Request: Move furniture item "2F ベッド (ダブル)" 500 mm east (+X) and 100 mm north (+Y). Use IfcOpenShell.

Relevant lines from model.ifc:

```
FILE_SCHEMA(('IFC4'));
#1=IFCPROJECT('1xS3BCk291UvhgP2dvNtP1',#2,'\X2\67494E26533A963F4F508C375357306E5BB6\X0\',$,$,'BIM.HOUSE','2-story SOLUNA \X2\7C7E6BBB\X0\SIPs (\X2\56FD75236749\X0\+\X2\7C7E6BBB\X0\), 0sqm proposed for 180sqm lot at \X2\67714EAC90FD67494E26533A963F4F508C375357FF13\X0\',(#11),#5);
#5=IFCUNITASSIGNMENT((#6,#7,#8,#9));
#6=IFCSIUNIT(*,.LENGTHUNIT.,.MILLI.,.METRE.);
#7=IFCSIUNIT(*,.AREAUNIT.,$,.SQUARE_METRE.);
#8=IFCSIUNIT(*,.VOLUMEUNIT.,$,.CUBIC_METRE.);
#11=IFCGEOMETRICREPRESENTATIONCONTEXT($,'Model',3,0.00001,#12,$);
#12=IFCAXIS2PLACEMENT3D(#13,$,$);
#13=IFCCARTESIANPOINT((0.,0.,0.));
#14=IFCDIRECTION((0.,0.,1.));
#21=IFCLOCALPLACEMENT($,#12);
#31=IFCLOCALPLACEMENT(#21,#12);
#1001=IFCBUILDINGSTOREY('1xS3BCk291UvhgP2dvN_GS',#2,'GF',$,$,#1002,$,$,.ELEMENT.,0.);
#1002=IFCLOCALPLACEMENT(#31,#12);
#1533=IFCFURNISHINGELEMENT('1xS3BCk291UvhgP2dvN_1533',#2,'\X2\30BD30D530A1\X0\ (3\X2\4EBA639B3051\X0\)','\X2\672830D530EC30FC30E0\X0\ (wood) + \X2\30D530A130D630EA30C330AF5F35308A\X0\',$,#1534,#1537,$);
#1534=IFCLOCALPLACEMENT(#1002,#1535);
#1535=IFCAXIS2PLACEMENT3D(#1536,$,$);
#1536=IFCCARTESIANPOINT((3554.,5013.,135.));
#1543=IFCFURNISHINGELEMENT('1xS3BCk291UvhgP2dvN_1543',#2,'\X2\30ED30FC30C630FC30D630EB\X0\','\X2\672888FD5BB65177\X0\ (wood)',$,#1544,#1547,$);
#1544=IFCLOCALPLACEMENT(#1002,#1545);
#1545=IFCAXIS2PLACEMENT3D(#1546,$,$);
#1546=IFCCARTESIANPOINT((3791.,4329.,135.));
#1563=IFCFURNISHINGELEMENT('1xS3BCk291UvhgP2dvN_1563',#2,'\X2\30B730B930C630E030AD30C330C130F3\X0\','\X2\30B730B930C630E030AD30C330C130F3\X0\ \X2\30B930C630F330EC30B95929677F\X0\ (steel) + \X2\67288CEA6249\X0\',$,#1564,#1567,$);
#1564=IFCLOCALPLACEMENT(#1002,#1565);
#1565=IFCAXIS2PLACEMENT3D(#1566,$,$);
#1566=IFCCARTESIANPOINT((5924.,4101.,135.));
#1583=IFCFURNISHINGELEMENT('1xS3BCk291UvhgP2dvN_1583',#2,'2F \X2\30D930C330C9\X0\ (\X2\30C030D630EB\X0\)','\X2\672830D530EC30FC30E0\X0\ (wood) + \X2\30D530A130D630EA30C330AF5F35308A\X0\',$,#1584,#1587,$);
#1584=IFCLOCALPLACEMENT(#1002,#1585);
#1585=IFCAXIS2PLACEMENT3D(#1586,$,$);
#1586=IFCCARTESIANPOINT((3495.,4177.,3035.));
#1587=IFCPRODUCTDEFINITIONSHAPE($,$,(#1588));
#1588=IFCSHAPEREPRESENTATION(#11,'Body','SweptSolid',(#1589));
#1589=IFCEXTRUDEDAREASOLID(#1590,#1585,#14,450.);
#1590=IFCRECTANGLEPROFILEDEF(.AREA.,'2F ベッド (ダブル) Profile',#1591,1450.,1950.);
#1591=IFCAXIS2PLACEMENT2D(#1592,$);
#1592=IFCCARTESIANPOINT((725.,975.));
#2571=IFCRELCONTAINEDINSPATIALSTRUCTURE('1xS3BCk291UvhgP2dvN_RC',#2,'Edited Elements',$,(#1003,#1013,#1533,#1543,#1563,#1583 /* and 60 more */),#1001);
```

```python
import ifcopenshell
import ifcopenshell.api.geometry
import ifcopenshell.util.placement
import ifcopenshell.util.unit

model = ifcopenshell.open("model.ifc")
unit_scale = ifcopenshell.util.unit.calculate_unit_scale(model)

item = model.by_guid("1xS3BCk291UvhgP2dvN_1583")
matrix = ifcopenshell.util.placement.get_local_placement(item.ObjectPlacement)
matrix[0, 3] += 0.5 / unit_scale
matrix[1, 3] += 0.1 / unit_scale
ifcopenshell.api.geometry.edit_object_placement(model, product=item, matrix=matrix, is_si=False)

print(ifcopenshell.util.placement.get_local_placement(item.ObjectPlacement).round(3) + 0.0)

model.write("model-out.ifc")
```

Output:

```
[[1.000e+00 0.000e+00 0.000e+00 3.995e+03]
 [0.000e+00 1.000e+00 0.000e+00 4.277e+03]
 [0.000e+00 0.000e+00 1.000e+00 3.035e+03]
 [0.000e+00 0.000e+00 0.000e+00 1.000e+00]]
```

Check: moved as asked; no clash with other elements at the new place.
